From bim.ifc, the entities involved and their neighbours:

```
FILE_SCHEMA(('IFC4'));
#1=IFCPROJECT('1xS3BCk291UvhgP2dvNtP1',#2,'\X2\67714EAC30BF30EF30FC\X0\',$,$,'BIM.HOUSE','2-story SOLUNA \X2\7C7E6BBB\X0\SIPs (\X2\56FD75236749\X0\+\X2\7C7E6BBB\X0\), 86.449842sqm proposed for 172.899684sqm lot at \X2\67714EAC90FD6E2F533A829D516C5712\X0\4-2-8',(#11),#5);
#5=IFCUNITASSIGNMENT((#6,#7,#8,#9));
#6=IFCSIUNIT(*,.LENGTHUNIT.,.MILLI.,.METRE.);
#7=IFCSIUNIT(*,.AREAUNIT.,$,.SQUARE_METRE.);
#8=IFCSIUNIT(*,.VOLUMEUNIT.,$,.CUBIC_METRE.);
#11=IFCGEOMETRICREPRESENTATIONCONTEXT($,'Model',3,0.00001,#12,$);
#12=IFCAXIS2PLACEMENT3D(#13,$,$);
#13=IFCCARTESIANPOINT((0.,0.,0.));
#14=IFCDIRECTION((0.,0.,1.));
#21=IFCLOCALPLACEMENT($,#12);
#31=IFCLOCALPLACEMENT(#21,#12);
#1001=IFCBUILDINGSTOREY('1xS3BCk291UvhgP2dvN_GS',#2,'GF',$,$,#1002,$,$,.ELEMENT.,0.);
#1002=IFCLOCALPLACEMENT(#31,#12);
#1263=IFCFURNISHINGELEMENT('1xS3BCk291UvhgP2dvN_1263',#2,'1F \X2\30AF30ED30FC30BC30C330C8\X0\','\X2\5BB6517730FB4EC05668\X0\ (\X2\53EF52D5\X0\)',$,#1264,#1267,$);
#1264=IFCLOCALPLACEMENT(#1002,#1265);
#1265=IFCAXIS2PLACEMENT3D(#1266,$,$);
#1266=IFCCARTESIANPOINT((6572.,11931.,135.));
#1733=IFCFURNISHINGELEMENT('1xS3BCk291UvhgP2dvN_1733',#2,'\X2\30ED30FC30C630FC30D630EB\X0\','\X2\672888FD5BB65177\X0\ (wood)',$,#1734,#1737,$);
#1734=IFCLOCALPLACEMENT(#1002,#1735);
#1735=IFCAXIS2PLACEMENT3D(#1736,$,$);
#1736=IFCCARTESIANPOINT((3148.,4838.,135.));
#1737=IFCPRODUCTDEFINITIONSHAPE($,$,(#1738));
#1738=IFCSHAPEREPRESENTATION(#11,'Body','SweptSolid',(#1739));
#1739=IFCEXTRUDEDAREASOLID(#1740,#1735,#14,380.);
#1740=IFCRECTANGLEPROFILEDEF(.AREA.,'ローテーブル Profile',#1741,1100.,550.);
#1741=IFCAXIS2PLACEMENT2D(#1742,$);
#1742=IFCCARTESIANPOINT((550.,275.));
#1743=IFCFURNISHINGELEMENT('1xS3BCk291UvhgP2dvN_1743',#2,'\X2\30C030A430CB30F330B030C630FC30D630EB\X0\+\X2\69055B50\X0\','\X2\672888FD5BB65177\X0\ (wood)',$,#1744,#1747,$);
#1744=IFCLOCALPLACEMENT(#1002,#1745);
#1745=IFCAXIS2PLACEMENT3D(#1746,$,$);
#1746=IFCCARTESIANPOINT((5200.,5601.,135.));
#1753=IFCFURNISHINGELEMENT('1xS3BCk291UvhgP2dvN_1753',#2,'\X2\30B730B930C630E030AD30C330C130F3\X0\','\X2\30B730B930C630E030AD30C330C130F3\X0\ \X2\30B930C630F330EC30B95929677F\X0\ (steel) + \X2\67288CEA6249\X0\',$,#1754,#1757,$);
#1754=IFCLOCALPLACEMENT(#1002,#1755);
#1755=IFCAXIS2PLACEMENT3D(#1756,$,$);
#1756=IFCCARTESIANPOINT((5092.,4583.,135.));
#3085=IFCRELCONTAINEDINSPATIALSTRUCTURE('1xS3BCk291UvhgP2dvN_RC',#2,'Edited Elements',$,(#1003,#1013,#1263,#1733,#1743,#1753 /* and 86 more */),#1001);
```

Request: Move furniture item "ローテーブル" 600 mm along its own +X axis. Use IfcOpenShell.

```python
import ifcopenshell
import ifcopenshell.api.geometry
import ifcopenshell.util.placement

model = ifcopenshell.open("bim.ifc")

item = model.by_id(1733)
matrix = ifcopenshell.util.placement.get_local_placement(item.ObjectPlacement)
matrix[:3, 3] += matrix[:3, 0] * 600.0
ifcopenshell.api.geometry.edit_object_placement(model, product=item, matrix=matrix, is_si=False)

print(ifcopenshell.util.placement.get_local_placement(item.ObjectPlacement).round(3) + 0.0)

model.write("bim_rev.ifc")
```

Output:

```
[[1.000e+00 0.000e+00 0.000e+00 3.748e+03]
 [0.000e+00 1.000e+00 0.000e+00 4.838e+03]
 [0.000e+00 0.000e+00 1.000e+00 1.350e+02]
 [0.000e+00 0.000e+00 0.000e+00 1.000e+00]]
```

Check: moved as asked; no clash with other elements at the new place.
